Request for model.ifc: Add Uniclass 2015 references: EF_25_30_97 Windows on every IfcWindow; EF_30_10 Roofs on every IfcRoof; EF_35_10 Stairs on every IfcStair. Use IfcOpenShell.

First a look at what the model holds.

```python
import ifcopenshell

model = ifcopenshell.open("model.ifc")
print(model.schema)
print("classifications:", [c.Name for c in model.by_type("IfcClassification")])
for ifc_class in ("IfcDoor", "IfcRoof", "IfcStair", "IfcWall", "IfcWindow"):
    print(ifc_class, len(model.by_type(ifc_class)))
```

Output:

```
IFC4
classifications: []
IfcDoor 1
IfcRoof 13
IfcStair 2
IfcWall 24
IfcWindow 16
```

```python
import ifcopenshell
import ifcopenshell.api.classification

model = ifcopenshell.open("model.ifc")

system = ifcopenshell.api.classification.add_classification(model, classification="Uniclass 2015")

codes = {
    "IfcWindow": ("EF_25_30_97", "Windows"),
    "IfcRoof": ("EF_30_10", "Roofs"),
    "IfcStair": ("EF_35_10", "Stairs"),
}
for ifc_class, (code, name) in codes.items():
    products = model.by_type(ifc_class)
    ifcopenshell.api.classification.add_reference(
        model, products=products, classification=system, identification=code, name=name
    )
    print(code, len(products))

model.write("model_updated.ifc")
```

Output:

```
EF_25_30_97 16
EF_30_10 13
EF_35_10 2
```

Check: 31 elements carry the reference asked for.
